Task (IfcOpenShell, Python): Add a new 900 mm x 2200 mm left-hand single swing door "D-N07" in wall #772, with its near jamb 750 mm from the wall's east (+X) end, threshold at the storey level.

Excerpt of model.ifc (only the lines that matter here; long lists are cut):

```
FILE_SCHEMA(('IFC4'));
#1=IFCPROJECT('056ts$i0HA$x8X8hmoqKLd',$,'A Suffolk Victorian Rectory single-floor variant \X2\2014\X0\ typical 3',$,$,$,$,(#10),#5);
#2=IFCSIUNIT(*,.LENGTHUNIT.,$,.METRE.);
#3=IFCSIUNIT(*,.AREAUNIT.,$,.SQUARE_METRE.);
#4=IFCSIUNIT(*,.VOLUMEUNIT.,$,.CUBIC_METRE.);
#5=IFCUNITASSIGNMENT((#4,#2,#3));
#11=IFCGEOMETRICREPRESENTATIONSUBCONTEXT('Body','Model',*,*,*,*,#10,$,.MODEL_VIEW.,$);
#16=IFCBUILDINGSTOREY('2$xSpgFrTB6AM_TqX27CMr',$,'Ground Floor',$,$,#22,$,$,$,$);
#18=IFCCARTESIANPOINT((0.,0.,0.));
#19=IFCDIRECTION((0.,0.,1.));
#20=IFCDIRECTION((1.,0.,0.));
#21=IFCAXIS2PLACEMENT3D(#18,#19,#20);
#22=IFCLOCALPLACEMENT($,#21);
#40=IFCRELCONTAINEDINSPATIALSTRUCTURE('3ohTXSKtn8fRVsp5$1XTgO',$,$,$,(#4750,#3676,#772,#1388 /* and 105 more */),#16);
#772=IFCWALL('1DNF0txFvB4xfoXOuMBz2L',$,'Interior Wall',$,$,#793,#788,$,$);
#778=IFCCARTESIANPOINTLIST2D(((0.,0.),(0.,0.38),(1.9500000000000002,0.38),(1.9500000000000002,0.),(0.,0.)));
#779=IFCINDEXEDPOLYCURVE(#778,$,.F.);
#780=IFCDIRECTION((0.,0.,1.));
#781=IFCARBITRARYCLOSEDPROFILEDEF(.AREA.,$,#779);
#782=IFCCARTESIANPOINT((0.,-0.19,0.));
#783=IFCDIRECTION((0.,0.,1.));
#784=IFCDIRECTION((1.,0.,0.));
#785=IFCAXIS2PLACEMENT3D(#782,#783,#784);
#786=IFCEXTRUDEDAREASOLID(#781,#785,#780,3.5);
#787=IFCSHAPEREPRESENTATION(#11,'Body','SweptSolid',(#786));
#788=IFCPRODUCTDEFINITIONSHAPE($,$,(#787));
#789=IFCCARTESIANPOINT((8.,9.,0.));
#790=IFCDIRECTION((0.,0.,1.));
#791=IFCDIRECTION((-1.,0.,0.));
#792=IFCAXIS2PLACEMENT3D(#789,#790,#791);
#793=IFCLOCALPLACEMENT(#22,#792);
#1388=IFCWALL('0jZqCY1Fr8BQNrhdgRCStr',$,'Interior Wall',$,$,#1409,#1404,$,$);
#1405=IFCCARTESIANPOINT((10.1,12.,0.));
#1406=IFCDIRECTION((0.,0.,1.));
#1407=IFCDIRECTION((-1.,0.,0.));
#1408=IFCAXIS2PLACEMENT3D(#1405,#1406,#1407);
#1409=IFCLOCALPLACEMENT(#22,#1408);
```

```python
import numpy as np
import ifcopenshell
import ifcopenshell.api.feature
import ifcopenshell.api.geometry
import ifcopenshell.api.root
import ifcopenshell.api.spatial
import ifcopenshell.geom
import ifcopenshell.util.element
import ifcopenshell.util.placement
import ifcopenshell.util.representation
import ifcopenshell.util.shape
import ifcopenshell.util.unit

model = ifcopenshell.open("model.ifc")
unit_scale = ifcopenshell.util.unit.calculate_unit_scale(model)
settings = ifcopenshell.geom.settings()


def volume(element):
    """Net volume in cubic metres, openings subtracted."""
    shape = ifcopenshell.geom.create_shape(settings, element)
    return ifcopenshell.util.shape.get_volume(shape.geometry)


wall = model.by_id(772)
storey = ifcopenshell.util.element.get_container(wall, ifc_class="IfcBuildingStorey")
context = ifcopenshell.util.representation.get_context(model, "Model", "Body", "MODEL_VIEW")
before = volume(wall)

width, height, from_end, sill = 0.9, 2.2, 0.75, 0.0  # metres

# The wall runs along its own X axis, and the end named is its -X end.
wall_shape = ifcopenshell.geom.create_shape(settings, wall)
x, y, z = ifcopenshell.util.shape.get_vertices(wall_shape.geometry).T
start = x.min() + from_end
face, thickness = float(y.min()), float(y.max() - y.min())
wall_matrix = ifcopenshell.util.placement.get_local_placement(wall.ObjectPlacement)
level = ifcopenshell.util.placement.get_local_placement(storey.ObjectPlacement)[2, 3]


def in_wall(x, y):
    """Placement at x, y metres in the wall's axes, at sill height."""
    matrix = wall_matrix.copy()
    matrix[:, 3] = wall_matrix @ np.array([x / unit_scale, y / unit_scale, 0.0, 1.0])
    matrix[2, 3] = level + sill / unit_scale
    return matrix


# Opening: a box that overshoots both wall faces by 50 mm.
opening = ifcopenshell.api.root.create_entity(model, ifc_class="IfcOpeningElement", predefined_type="OPENING")
box = ifcopenshell.api.geometry.add_wall_representation(
    model, context=context, length=width, height=height, thickness=thickness + 0.1
)
ifcopenshell.api.geometry.assign_representation(model, product=opening, representation=box)
ifcopenshell.api.geometry.edit_object_placement(model, product=opening, matrix=in_wall(start, face - 0.05), is_si=False)
ifcopenshell.api.feature.add_feature(model, feature=opening, element=wall)

door = ifcopenshell.api.root.create_entity(model, ifc_class="IfcDoor", name="D-N07", predefined_type="DOOR")
door.OverallWidth, door.OverallHeight = width / unit_scale, height / unit_scale
door.OperationType = "SINGLE_SWING_LEFT"
body = ifcopenshell.api.geometry.add_door_representation(
    model,
    context=context,
    overall_width=door.OverallWidth,
    overall_height=door.OverallHeight,
    operation_type="SINGLE_SWING_LEFT",
    lining_properties={"LiningDepth": thickness / unit_scale, "ThresholdDepth": thickness / unit_scale},
)
ifcopenshell.api.geometry.assign_representation(model, product=door, representation=body)
ifcopenshell.api.spatial.assign_container(model, products=[door], relating_structure=storey)
ifcopenshell.api.feature.add_filling(model, opening=opening, element=door)

# The lining spans the wall, so the door starts at the wall face.
ifcopenshell.api.geometry.edit_object_placement(model, product=door, matrix=in_wall(start, face), is_si=False)

after = volume(wall)

print(f"wall volume {before:.3f} -> {after:.3f} m3")

model.write("model-out.ifc")
```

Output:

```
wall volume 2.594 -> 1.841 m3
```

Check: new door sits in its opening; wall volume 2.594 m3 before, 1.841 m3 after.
